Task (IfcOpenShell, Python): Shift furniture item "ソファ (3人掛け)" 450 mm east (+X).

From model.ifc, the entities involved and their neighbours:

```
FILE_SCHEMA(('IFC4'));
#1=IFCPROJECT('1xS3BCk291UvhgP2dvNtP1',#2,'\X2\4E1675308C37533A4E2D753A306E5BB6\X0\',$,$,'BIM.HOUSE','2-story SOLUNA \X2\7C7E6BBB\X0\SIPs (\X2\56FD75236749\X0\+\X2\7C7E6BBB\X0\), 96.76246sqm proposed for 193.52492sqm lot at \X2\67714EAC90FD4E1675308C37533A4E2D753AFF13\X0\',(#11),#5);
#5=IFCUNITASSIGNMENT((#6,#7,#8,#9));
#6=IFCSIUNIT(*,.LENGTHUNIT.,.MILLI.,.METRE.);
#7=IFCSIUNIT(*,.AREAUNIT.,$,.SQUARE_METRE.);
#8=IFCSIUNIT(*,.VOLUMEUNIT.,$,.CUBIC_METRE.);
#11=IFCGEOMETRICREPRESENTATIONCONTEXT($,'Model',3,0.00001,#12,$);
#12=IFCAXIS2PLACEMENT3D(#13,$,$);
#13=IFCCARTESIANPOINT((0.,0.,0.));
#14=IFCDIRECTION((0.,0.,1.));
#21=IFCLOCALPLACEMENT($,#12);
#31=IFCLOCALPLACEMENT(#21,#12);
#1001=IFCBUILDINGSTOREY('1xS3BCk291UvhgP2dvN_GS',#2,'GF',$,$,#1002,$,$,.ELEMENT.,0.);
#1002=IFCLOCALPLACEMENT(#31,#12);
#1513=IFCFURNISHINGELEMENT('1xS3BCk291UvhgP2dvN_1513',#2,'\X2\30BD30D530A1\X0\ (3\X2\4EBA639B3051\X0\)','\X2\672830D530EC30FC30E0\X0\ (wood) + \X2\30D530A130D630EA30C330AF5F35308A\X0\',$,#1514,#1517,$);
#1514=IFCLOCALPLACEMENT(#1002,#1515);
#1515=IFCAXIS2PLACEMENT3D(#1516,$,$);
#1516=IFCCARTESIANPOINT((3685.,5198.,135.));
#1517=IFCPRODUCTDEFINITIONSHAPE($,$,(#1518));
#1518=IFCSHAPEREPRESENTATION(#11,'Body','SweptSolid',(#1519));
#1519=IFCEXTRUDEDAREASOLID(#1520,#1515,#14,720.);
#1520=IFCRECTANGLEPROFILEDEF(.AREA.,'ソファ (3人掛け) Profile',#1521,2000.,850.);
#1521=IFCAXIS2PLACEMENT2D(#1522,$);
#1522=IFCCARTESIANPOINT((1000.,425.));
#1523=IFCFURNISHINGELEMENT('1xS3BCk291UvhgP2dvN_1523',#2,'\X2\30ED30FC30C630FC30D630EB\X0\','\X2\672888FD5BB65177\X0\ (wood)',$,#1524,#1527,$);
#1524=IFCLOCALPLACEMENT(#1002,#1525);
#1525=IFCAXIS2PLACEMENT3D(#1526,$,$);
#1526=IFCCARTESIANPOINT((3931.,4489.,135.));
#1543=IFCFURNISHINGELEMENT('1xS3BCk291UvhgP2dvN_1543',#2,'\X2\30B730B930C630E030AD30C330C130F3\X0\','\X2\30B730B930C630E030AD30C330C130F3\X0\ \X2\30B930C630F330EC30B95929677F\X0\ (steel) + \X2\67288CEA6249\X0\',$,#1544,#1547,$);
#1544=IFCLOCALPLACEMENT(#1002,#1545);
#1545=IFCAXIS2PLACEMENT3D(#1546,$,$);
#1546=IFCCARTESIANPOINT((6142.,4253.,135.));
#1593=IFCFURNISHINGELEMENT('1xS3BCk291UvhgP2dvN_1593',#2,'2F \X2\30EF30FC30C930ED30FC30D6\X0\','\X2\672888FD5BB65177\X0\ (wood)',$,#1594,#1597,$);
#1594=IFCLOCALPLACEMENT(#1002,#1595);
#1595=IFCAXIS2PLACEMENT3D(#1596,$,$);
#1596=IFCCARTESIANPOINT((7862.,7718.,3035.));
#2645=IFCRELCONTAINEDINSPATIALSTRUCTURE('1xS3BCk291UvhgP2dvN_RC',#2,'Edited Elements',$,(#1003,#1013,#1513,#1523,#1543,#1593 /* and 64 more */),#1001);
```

```python
import ifcopenshell
import ifcopenshell.api.geometry
import ifcopenshell.util.placement

model = ifcopenshell.open("model.ifc")

item = model.by_guid("1xS3BCk291UvhgP2dvN_1513")
matrix = ifcopenshell.util.placement.get_local_placement(item.ObjectPlacement)
matrix[0, 3] += 450.0
ifcopenshell.api.geometry.edit_object_placement(model, product=item, matrix=matrix, is_si=False)

print(ifcopenshell.util.placement.get_local_placement(item.ObjectPlacement).round(3) + 0.0)

model.write("model_v2.ifc")
```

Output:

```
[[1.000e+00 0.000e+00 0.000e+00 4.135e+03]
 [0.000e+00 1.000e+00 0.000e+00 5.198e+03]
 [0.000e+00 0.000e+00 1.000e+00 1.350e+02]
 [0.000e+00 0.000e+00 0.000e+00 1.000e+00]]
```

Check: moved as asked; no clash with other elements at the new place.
